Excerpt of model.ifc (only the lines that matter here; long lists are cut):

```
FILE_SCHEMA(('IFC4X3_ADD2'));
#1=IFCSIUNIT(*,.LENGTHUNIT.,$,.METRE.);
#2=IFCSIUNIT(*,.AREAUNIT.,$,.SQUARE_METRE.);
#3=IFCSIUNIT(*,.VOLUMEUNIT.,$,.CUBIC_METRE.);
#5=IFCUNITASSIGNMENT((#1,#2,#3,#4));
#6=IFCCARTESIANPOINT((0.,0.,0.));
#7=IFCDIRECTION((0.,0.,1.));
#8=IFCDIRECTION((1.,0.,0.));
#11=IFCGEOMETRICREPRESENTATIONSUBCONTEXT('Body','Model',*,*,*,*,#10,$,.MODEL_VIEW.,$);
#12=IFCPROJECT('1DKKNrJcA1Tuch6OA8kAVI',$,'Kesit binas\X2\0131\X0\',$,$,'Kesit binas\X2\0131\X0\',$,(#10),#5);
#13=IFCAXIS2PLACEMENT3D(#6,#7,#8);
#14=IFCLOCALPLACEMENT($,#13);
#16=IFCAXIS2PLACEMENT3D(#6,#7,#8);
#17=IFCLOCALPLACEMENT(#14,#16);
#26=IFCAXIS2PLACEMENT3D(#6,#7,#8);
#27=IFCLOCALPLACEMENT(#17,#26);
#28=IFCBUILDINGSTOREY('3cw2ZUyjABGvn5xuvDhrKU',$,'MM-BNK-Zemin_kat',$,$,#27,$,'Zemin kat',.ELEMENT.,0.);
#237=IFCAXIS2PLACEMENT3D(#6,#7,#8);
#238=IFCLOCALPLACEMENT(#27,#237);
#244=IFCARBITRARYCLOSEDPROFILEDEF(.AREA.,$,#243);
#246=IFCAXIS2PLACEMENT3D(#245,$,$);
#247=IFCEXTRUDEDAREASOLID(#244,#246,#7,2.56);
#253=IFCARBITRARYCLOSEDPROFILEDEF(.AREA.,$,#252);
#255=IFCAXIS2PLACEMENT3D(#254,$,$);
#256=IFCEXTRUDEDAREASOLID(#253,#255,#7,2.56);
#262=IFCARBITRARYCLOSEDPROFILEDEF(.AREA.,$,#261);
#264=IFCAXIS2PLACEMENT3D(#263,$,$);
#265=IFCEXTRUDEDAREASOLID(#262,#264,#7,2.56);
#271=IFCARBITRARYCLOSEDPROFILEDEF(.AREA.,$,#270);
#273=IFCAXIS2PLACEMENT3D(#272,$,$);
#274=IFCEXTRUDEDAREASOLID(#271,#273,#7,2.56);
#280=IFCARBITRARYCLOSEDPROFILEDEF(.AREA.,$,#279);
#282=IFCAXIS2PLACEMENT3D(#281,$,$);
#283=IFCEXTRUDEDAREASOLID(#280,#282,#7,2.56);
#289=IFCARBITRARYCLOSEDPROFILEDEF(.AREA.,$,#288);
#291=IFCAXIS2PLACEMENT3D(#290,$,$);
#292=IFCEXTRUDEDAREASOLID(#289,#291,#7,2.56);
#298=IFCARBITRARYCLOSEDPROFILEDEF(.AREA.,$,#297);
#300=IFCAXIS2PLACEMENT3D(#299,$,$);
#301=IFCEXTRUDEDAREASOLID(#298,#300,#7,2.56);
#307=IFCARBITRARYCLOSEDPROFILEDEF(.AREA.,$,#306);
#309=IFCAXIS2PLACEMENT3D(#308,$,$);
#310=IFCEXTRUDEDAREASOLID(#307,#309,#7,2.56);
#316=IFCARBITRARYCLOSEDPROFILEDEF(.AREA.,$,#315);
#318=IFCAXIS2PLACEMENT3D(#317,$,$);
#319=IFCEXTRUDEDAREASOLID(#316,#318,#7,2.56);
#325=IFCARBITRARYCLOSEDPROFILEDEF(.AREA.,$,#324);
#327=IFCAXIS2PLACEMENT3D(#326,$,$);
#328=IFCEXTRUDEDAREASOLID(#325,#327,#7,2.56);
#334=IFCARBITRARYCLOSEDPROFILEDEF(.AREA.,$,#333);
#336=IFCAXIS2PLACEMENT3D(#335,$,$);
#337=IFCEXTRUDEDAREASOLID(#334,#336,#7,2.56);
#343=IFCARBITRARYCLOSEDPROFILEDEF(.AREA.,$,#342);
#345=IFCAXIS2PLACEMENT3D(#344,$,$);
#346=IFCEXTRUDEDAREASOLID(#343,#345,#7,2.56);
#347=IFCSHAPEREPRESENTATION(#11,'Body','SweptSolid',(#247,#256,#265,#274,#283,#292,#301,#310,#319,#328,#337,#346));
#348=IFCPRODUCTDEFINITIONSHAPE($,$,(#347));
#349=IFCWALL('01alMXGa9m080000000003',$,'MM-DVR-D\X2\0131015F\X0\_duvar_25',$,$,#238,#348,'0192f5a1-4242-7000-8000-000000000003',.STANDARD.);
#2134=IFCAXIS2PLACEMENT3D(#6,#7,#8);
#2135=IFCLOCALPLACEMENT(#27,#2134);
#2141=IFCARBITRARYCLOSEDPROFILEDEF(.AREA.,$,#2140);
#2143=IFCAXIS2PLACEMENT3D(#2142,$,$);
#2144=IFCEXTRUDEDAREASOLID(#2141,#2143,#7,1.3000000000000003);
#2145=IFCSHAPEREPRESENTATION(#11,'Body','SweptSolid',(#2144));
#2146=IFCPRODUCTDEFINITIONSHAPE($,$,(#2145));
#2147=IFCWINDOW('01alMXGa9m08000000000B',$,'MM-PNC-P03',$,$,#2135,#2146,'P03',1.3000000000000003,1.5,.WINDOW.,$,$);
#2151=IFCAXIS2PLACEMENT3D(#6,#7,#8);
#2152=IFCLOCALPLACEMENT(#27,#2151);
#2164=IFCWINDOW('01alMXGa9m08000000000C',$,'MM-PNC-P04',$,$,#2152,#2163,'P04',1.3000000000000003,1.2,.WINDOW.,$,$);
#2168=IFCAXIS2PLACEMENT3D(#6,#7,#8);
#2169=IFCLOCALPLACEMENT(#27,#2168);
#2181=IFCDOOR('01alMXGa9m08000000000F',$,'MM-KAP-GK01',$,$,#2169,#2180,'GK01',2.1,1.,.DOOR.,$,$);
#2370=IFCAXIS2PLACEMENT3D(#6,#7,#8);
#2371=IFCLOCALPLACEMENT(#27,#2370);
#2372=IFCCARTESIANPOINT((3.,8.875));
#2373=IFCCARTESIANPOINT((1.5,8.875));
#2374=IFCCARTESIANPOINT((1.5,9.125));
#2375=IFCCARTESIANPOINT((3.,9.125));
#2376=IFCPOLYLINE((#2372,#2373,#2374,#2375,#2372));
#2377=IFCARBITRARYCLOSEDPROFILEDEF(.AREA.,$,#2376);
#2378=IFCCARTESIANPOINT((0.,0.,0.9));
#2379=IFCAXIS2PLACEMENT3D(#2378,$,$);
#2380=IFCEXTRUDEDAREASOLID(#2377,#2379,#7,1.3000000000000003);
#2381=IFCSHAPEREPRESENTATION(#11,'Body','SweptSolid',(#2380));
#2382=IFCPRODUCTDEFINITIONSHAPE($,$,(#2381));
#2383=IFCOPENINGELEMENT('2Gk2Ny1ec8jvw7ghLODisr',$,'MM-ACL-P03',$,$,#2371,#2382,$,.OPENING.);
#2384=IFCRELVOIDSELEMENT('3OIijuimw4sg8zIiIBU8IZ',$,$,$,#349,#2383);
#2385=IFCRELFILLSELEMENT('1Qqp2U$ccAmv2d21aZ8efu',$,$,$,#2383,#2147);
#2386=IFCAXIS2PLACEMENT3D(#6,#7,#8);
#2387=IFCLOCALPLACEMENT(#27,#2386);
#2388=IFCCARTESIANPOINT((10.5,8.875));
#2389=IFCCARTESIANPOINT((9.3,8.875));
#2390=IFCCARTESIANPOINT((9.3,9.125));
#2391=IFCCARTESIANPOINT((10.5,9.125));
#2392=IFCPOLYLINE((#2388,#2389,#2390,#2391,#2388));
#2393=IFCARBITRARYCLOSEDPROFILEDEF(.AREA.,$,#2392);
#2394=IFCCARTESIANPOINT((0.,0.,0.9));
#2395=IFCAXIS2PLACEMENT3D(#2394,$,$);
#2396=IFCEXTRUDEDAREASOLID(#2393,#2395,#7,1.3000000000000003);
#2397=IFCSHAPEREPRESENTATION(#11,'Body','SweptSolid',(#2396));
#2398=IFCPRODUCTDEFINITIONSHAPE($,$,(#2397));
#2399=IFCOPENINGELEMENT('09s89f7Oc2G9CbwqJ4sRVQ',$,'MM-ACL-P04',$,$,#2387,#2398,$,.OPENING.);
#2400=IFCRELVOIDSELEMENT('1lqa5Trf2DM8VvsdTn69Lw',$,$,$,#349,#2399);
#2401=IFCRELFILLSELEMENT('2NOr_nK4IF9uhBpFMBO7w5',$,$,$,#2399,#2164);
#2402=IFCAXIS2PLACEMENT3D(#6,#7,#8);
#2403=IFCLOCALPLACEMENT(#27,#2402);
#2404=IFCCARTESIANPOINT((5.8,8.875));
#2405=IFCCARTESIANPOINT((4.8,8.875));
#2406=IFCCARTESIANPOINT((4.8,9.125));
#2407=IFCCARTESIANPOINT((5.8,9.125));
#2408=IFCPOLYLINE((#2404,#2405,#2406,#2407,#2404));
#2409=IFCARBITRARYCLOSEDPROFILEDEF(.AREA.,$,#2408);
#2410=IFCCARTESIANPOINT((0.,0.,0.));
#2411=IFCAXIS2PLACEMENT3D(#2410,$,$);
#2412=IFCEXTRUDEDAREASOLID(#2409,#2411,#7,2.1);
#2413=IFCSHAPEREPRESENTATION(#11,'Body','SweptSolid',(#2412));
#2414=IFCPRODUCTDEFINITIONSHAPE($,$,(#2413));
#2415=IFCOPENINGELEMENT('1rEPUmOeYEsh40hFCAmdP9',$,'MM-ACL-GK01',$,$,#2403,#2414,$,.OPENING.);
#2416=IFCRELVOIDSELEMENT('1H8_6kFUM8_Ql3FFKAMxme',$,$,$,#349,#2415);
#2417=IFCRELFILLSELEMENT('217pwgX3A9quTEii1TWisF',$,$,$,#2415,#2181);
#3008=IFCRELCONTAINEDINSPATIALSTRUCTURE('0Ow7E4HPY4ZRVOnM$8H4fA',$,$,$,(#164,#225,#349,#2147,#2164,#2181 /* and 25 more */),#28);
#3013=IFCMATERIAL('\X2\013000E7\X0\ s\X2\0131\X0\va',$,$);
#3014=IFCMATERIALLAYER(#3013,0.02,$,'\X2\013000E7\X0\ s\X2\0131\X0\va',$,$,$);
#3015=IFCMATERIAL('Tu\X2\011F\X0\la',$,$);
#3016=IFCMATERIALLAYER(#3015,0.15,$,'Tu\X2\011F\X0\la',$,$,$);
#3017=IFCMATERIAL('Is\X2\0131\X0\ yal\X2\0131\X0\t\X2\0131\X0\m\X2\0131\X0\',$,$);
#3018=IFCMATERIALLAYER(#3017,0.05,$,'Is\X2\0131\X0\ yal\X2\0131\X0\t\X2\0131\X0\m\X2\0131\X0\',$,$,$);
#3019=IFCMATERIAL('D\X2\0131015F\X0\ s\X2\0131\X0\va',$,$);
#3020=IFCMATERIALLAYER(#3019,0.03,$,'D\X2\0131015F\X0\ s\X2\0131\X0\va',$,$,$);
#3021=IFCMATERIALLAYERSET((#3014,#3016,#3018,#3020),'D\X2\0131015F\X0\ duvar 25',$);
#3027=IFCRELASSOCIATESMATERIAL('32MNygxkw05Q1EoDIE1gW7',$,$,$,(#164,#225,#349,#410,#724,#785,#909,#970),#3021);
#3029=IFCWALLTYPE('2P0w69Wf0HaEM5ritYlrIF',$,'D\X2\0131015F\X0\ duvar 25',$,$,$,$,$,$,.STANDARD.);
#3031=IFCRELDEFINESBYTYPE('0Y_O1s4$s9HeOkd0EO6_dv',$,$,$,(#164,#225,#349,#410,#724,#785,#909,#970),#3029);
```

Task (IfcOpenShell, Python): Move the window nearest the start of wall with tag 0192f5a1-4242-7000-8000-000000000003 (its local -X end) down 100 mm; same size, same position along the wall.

```python
import numpy as np
import ifcopenshell
import ifcopenshell.api.geometry
import ifcopenshell.util.placement
import ifcopenshell.util.unit

model = ifcopenshell.open("model.ifc")
unit_scale = ifcopenshell.util.unit.calculate_unit_scale(model)

window = model.by_id(2147)
opening = window.FillsVoids[0].RelatingOpeningElement
dz = -0.1

shift = np.array([0.0, 0.0, dz])
# The window is not placed relative to its opening, so move both.
for product in (opening, window):
    matrix = ifcopenshell.util.placement.get_local_placement(product.ObjectPlacement)
    matrix[:3, 3] += shift
    ifcopenshell.api.geometry.edit_object_placement(model, product=product, matrix=matrix, is_si=False)

print(f"moved by {dz * unit_scale:+.3f} m")

model.write("model-out.ifc")
```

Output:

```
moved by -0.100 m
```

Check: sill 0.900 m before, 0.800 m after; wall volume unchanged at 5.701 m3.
